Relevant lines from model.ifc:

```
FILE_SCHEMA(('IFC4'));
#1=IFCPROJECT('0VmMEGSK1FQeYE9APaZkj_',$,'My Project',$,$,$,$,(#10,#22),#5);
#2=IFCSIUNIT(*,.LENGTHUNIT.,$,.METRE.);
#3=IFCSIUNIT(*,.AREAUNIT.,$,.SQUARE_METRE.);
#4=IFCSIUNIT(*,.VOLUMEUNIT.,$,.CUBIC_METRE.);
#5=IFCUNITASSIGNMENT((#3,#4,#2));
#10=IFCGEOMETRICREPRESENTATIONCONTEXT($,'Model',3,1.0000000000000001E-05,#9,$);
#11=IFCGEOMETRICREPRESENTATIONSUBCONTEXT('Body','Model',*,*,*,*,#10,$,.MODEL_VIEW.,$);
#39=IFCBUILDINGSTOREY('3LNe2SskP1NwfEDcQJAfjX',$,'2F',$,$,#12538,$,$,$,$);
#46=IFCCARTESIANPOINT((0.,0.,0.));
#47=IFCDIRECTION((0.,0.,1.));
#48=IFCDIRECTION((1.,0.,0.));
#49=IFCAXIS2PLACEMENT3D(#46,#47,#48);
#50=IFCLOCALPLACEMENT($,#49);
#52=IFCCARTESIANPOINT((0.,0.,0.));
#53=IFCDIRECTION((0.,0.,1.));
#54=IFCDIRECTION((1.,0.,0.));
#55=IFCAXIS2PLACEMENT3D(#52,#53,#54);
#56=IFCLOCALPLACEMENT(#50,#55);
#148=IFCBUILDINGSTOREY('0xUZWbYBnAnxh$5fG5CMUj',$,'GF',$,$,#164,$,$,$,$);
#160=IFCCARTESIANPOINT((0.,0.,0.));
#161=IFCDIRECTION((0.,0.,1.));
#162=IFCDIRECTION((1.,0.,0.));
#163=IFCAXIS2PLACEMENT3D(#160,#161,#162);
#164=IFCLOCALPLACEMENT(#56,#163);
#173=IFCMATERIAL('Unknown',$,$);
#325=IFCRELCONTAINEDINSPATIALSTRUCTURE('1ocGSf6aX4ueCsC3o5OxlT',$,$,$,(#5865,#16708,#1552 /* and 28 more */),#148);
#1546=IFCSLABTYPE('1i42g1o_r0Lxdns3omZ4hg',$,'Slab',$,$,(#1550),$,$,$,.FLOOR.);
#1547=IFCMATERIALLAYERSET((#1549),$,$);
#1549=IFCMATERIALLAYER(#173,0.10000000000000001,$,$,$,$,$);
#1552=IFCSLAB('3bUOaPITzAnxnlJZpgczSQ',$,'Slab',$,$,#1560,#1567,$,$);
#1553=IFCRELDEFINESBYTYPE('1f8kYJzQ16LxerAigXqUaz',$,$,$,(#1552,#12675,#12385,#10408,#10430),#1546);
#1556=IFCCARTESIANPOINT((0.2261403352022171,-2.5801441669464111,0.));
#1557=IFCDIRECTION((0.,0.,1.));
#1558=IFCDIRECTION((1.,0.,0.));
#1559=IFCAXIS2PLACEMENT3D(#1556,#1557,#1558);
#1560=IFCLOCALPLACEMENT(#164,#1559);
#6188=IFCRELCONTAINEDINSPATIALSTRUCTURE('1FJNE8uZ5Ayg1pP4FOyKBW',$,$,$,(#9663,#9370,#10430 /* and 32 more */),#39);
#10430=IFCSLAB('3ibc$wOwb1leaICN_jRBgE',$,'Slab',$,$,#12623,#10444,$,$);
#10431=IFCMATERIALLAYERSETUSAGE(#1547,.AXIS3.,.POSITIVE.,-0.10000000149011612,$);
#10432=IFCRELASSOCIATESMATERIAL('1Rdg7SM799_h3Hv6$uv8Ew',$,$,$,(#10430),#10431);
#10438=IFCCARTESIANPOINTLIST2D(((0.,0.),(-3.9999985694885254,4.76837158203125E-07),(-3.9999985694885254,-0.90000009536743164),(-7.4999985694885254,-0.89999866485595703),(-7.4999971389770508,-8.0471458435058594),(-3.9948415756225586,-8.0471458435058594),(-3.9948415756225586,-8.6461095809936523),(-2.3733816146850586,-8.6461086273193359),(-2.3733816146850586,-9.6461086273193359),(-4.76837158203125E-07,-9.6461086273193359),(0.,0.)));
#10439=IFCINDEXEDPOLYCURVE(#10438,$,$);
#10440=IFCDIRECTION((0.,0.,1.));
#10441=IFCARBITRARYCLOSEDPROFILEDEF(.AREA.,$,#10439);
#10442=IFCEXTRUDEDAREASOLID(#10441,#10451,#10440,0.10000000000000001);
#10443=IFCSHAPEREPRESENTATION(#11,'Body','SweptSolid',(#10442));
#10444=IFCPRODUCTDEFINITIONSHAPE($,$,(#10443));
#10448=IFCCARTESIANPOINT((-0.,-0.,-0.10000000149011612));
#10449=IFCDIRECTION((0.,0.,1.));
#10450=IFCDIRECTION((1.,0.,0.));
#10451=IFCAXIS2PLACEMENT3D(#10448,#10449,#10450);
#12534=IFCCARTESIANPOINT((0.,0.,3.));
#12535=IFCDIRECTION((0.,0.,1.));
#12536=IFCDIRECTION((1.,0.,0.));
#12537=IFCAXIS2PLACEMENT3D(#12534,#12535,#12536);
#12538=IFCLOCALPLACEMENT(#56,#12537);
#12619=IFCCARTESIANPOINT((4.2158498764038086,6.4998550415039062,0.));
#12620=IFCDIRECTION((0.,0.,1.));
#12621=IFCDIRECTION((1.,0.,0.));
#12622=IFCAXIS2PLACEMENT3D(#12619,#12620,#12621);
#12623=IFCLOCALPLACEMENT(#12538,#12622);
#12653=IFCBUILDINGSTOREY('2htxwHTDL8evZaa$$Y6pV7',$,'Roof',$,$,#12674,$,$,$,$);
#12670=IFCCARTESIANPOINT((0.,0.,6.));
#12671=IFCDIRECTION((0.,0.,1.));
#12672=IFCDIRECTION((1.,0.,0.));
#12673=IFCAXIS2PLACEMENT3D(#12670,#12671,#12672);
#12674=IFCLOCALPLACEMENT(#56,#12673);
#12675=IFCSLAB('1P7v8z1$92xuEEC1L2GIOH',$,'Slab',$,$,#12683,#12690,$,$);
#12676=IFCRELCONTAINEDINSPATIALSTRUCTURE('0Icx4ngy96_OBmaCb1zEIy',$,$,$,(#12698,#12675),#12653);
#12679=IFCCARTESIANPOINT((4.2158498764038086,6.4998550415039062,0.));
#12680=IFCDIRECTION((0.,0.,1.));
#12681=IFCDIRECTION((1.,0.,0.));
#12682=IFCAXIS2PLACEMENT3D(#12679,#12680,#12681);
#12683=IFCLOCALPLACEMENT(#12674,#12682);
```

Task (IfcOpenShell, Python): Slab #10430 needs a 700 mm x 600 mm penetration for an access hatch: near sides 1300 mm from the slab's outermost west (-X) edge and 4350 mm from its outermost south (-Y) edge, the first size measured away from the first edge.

```python
import numpy as np
import ifcopenshell
import ifcopenshell.api.feature
import ifcopenshell.api.geometry
import ifcopenshell.api.root
import ifcopenshell.geom
import ifcopenshell.util.placement
import ifcopenshell.util.representation
import ifcopenshell.util.shape
import ifcopenshell.util.unit

model = ifcopenshell.open("model.ifc")
unit_scale = ifcopenshell.util.unit.calculate_unit_scale(model)
settings = ifcopenshell.geom.settings()


def volume(element):
    """Net volume in cubic metres, openings subtracted."""
    shape = ifcopenshell.geom.create_shape(settings, element)
    return ifcopenshell.util.shape.get_volume(shape.geometry)


slab = model.by_guid("3ibc$wOwb1leaICN_jRBgE")
before = volume(slab)

# Extent in the slab's own axes, in metres. The edges named are its -X and -Y sides.
slab_shape = ifcopenshell.geom.create_shape(settings, slab)
vertices = ifcopenshell.util.shape.get_vertices(slab_shape.geometry)
x_min, y_min, bottom = vertices.min(axis=0)
top = vertices[:, 2].max()

opening = ifcopenshell.api.root.create_entity(model, ifc_class="IfcOpeningElement", name="Access hatch opening", predefined_type="OPENING")
context = ifcopenshell.util.representation.get_context(model, "Model", "Body", "MODEL_VIEW")
width, depth = 0.7, 0.6
outline = [(0.0, 0.0), (width, 0.0), (width, depth), (0.0, depth), (0.0, 0.0)]
# Overshoot both faces by 50 mm so the cut is clean.
shape = ifcopenshell.api.geometry.add_slab_representation(
    model, context=context, depth=top - bottom + 0.1, polyline=outline
)
ifcopenshell.api.geometry.assign_representation(model, product=opening, representation=shape)

matrix = ifcopenshell.util.placement.get_local_placement(slab.ObjectPlacement)
matrix[:, 3] = matrix @ np.append(np.array([x_min + 1.3, y_min + 4.35, bottom - 0.05]) / unit_scale, 1.0)
ifcopenshell.api.geometry.edit_object_placement(model, product=opening, matrix=matrix, is_si=False)
ifcopenshell.api.feature.add_feature(model, feature=opening, element=slab)

after = volume(slab)

print(f"slab volume {before:.3f} -> {after:.3f} m3")

model.write("model_edited.ifc")
```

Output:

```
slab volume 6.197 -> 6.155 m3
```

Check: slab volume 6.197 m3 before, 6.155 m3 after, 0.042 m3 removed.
